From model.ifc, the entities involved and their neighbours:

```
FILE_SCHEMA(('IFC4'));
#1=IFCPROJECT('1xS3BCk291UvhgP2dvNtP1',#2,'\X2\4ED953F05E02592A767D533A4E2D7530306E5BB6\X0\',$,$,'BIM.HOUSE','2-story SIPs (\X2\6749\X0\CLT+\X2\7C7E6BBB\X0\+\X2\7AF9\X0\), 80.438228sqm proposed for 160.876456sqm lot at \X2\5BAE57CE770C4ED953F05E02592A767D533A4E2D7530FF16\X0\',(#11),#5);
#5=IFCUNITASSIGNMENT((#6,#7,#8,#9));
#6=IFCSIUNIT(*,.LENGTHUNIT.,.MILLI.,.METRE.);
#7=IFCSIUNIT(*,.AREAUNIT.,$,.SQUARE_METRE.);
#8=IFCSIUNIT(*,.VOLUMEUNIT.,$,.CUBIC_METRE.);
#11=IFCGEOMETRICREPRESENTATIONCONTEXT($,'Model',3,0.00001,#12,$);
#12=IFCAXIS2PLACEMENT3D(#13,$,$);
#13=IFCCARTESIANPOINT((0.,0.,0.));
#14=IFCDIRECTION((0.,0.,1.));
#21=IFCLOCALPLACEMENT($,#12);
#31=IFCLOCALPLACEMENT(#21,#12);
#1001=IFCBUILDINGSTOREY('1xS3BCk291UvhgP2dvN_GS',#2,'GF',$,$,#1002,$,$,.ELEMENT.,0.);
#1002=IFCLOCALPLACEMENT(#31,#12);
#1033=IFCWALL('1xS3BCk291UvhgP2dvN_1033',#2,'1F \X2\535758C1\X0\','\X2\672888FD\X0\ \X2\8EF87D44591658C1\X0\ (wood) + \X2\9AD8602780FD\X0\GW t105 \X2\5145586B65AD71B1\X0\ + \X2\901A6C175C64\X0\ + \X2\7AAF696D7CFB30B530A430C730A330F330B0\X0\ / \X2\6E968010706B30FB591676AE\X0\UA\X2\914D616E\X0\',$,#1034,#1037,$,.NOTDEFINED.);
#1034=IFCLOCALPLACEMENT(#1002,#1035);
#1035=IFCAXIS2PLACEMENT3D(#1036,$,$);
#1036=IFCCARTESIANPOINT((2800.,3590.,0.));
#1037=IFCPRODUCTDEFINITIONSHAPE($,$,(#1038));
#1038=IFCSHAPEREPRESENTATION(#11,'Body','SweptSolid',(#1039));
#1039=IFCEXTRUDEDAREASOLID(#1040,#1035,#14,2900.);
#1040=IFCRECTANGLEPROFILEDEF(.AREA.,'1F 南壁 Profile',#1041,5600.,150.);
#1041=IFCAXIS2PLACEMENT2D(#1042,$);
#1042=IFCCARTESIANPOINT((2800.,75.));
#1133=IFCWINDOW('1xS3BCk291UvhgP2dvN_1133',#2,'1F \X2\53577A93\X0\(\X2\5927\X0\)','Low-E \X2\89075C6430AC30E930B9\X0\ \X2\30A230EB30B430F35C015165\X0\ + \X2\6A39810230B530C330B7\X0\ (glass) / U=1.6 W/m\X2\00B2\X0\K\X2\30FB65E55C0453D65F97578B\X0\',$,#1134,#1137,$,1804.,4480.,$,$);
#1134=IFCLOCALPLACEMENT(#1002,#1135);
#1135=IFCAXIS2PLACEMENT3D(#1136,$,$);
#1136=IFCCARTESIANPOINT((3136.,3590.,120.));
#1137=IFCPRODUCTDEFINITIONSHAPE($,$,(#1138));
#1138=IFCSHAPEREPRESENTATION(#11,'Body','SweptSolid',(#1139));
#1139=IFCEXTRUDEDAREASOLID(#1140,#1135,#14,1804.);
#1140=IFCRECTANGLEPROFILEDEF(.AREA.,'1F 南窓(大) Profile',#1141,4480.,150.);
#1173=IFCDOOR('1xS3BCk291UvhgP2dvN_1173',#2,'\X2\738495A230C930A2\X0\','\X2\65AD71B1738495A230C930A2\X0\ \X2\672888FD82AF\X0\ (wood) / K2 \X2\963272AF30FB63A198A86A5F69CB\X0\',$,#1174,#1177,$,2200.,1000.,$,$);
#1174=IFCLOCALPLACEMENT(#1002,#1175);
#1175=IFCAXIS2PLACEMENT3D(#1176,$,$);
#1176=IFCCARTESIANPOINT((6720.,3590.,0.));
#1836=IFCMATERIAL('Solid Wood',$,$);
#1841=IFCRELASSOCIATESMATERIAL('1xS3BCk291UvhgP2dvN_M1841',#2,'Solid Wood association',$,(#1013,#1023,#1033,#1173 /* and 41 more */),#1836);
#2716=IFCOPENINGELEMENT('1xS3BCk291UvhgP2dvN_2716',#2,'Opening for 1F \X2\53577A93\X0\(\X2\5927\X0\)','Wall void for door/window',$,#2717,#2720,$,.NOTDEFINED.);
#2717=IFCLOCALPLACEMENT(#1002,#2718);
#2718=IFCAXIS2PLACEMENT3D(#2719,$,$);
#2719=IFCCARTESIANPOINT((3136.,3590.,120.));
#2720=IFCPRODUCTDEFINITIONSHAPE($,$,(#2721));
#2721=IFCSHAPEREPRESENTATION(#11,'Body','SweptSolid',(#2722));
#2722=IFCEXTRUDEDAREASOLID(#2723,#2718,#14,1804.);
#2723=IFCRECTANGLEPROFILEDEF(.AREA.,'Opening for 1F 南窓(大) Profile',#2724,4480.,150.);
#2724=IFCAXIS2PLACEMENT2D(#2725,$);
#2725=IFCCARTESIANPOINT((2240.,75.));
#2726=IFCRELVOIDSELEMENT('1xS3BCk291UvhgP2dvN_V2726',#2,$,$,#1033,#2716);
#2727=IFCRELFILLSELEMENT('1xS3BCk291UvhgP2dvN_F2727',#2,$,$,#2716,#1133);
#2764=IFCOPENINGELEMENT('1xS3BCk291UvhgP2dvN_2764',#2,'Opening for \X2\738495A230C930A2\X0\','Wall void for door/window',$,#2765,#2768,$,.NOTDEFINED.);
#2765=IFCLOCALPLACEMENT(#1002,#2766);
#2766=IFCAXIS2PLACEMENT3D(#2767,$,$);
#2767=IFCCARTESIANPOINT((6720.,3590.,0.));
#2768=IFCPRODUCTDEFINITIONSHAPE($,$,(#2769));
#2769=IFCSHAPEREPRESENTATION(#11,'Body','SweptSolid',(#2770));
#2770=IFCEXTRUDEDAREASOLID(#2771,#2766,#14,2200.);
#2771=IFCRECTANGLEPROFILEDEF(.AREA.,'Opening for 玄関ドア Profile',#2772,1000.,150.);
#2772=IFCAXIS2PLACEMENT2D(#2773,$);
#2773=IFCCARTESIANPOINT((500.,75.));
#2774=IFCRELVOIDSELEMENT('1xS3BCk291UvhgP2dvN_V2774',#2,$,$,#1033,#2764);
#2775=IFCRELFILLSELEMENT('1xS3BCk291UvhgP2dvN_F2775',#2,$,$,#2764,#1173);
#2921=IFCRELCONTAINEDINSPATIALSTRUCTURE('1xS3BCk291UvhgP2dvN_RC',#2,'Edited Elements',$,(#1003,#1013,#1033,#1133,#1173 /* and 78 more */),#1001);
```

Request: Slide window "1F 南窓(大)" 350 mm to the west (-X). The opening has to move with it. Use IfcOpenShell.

```python
import ifcopenshell
import ifcopenshell.api.geometry
import ifcopenshell.util.placement
import ifcopenshell.util.unit

model = ifcopenshell.open("model.ifc")
unit_scale = ifcopenshell.util.unit.calculate_unit_scale(model)

window = model.by_guid("1xS3BCk291UvhgP2dvN_1133")
opening = window.FillsVoids[0].RelatingOpeningElement
wall = opening.VoidsElements[0].RelatingBuildingElement

wall_matrix = ifcopenshell.util.placement.get_local_placement(wall.ObjectPlacement)
shift = wall_matrix[:3, 0] * -0.35 / unit_scale
before = ifcopenshell.util.placement.get_local_placement(window.ObjectPlacement)[:3, 3].copy()

# The window is not placed relative to its opening, so move both.
for product in (opening, window):
    matrix = ifcopenshell.util.placement.get_local_placement(product.ObjectPlacement)
    matrix[:3, 3] += shift
    ifcopenshell.api.geometry.edit_object_placement(model, product=product, matrix=matrix, is_si=False)

after = ifcopenshell.util.placement.get_local_placement(window.ObjectPlacement)[:3, 3]
print("window moved by", (after - before).round(3) + 0.0)

model.write("model-out.ifc")
```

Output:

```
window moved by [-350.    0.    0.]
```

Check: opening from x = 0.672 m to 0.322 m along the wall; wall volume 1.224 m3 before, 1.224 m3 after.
